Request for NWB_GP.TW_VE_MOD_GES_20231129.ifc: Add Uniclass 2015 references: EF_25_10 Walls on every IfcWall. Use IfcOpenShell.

First a look at what the model holds.

```python
import ifcopenshell

model = ifcopenshell.open("NWB_GP.TW_VE_MOD_GES_20231129.ifc")
print(model.schema)
print("classifications:", [c.Name for c in model.by_type("IfcClassification")])
for ifc_class in ("IfcDoor", "IfcRoof", "IfcStair", "IfcWall", "IfcWindow"):
    print(ifc_class, len(model.by_type(ifc_class)))
```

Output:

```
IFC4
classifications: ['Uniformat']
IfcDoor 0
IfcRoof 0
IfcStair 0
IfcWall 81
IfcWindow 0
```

```python
import ifcopenshell
import ifcopenshell.api.classification

model = ifcopenshell.open("NWB_GP.TW_VE_MOD_GES_20231129.ifc")

system = ifcopenshell.api.classification.add_classification(model, classification="Uniclass 2015")

codes = {
    "IfcWall": ("EF_25_10", "Walls"),
}
for ifc_class, (code, name) in codes.items():
    products = model.by_type(ifc_class)
    ifcopenshell.api.classification.add_reference(
        model, products=products, classification=system, identification=code, name=name
    )
    print(code, len(products))

model.write("NWB_GP.TW_VE_MOD_GES_20231129_updated.ifc")
```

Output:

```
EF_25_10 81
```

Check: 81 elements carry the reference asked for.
